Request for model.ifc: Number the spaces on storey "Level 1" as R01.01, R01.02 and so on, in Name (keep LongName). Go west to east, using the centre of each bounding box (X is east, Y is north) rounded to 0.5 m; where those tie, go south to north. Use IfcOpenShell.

First a look at what the model holds.

```python
import ifcopenshell
import ifcopenshell.util.element
import ifcopenshell.util.placement

model = ifcopenshell.open("model.ifc")
print(model.schema)
storey = next(s for s in model.by_type("IfcBuildingStorey") if s.Name == "Level 1")
spaces = [e for e in ifcopenshell.util.element.get_decomposition(storey) if e.is_a("IfcSpace")]
for e in sorted(spaces, key=lambda e: e.id()):
    origin = ifcopenshell.util.placement.get_local_placement(e.ObjectPlacement)[:3, 3]
    print(e.id(), e.Name, e.LongName, origin.round(2) + 0.0, sep=" | ")
```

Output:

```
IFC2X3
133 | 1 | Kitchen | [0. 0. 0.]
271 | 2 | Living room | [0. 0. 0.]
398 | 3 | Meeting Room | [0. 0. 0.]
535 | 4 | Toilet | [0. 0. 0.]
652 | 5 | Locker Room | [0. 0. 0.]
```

```python
import ifcopenshell
import ifcopenshell.geom
import ifcopenshell.util.element
import ifcopenshell.util.shape

model = ifcopenshell.open("model.ifc")
settings = ifcopenshell.geom.settings()
settings.set("use-world-coords", True)


def centre(element):
    shape = ifcopenshell.geom.create_shape(settings, element)
    return ifcopenshell.util.shape.get_bbox_centroid(shape.geometry)


storey = next(s for s in model.by_type("IfcBuildingStorey") if s.Name == "Level 1")
spaces = [e for e in ifcopenshell.util.element.get_decomposition(storey) if e.is_a("IfcSpace")]

# Insertion points can sit at a corner or the storey origin, so sort by the geometry (in metres).
centres = {e: centre(e) for e in spaces}
spaces.sort(key=lambda e: (round(centres[e][0] / 0.5), centres[e][1]))

for i, e in enumerate(spaces, start=1):
    number = f"R01.{i:02d}"
    e.Name = number
    print(e.id(), number)

model.write("model_edited.ifc")
```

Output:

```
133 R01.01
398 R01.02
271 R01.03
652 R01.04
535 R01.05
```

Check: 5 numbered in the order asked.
